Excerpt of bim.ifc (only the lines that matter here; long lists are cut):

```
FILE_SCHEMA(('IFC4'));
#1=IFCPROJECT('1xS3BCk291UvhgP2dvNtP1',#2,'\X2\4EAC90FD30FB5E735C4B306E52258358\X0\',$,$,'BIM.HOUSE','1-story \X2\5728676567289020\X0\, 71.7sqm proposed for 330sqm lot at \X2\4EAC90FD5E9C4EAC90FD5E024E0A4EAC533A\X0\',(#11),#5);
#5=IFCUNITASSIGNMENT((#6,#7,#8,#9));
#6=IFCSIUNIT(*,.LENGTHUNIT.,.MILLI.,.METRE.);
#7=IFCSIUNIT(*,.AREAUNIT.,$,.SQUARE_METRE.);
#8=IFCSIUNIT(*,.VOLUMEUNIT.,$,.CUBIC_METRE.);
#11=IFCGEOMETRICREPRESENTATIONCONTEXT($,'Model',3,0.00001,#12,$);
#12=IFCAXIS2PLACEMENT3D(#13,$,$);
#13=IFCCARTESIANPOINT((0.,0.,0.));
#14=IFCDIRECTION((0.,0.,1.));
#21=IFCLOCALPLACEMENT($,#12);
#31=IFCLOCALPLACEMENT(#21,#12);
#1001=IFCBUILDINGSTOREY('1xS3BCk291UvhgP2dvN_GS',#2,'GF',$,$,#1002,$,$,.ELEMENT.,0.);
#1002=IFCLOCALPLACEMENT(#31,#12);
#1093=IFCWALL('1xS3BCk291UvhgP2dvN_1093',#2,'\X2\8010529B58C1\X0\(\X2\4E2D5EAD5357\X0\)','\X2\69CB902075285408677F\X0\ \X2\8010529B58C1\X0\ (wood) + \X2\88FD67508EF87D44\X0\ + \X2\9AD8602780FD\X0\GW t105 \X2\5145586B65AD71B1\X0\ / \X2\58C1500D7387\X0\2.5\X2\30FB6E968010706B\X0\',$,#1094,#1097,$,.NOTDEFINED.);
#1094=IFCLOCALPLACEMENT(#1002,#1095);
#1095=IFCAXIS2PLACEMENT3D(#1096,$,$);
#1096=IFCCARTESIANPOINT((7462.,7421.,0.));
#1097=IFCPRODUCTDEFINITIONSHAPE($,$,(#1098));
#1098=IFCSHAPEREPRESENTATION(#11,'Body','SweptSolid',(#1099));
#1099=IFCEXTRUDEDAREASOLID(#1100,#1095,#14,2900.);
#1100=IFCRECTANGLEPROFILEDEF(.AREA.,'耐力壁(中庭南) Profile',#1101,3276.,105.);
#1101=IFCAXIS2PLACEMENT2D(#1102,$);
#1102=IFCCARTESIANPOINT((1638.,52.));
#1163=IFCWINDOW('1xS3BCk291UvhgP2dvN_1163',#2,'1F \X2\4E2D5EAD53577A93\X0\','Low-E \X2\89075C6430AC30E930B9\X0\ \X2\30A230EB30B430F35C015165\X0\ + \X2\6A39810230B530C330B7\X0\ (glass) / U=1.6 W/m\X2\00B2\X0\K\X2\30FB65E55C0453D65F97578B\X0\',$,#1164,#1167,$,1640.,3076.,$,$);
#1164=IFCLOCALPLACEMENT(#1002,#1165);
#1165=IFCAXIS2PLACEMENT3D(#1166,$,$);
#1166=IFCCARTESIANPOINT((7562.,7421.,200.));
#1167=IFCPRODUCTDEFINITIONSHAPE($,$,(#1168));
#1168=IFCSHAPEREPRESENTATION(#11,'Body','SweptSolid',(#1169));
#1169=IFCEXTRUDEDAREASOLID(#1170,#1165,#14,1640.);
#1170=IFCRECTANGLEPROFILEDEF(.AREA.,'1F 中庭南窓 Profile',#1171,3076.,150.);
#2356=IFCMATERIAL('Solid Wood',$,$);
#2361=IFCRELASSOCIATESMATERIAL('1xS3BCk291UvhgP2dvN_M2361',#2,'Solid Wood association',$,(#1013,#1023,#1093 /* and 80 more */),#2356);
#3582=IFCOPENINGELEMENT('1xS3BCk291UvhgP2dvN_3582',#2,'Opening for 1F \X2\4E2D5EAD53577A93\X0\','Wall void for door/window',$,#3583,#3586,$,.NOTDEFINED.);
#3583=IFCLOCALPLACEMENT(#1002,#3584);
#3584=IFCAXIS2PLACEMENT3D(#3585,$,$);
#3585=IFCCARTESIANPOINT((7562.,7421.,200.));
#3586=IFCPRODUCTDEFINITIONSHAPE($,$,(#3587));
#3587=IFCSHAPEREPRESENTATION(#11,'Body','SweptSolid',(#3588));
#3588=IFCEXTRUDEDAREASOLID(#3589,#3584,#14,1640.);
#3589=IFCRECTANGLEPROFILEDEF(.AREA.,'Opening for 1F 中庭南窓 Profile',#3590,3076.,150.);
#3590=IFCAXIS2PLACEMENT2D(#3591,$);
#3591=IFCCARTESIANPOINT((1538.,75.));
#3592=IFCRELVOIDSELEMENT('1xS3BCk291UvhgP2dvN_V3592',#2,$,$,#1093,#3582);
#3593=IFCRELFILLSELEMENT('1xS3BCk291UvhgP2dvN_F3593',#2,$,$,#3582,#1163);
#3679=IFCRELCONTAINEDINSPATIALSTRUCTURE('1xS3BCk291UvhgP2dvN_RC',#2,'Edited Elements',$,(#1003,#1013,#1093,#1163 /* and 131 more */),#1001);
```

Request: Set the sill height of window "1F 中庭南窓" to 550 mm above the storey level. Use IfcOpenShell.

```python
import numpy as np
import ifcopenshell
import ifcopenshell.api.geometry
import ifcopenshell.geom
import ifcopenshell.util.element
import ifcopenshell.util.placement
import ifcopenshell.util.shape
import ifcopenshell.util.unit

model = ifcopenshell.open("bim.ifc")
unit_scale = ifcopenshell.util.unit.calculate_unit_scale(model)

window = model.by_guid("1xS3BCk291UvhgP2dvN_1163")
opening = window.FillsVoids[0].RelatingOpeningElement
storey = ifcopenshell.util.element.get_container(window, ifc_class="IfcBuildingStorey")
level = ifcopenshell.util.placement.get_local_placement(storey.ObjectPlacement)[2, 3]

# The opening's origin need not be at the sill, so measure its lowest point.
shape = ifcopenshell.geom.create_shape(ifcopenshell.geom.settings(), opening)
bottom = ifcopenshell.util.shape.get_shape_bottom_elevation(shape, shape.geometry) / unit_scale
dz = level + 550.0 - bottom

shift = np.array([0.0, 0.0, dz])
# The window is not placed relative to its opening, so move both.
for product in (opening, window):
    matrix = ifcopenshell.util.placement.get_local_placement(product.ObjectPlacement)
    matrix[:3, 3] += shift
    ifcopenshell.api.geometry.edit_object_placement(model, product=product, matrix=matrix, is_si=False)

print(f"moved by {dz * unit_scale:+.3f} m")

model.write("bim_v2.ifc")
```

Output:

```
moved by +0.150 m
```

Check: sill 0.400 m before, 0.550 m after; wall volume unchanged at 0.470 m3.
